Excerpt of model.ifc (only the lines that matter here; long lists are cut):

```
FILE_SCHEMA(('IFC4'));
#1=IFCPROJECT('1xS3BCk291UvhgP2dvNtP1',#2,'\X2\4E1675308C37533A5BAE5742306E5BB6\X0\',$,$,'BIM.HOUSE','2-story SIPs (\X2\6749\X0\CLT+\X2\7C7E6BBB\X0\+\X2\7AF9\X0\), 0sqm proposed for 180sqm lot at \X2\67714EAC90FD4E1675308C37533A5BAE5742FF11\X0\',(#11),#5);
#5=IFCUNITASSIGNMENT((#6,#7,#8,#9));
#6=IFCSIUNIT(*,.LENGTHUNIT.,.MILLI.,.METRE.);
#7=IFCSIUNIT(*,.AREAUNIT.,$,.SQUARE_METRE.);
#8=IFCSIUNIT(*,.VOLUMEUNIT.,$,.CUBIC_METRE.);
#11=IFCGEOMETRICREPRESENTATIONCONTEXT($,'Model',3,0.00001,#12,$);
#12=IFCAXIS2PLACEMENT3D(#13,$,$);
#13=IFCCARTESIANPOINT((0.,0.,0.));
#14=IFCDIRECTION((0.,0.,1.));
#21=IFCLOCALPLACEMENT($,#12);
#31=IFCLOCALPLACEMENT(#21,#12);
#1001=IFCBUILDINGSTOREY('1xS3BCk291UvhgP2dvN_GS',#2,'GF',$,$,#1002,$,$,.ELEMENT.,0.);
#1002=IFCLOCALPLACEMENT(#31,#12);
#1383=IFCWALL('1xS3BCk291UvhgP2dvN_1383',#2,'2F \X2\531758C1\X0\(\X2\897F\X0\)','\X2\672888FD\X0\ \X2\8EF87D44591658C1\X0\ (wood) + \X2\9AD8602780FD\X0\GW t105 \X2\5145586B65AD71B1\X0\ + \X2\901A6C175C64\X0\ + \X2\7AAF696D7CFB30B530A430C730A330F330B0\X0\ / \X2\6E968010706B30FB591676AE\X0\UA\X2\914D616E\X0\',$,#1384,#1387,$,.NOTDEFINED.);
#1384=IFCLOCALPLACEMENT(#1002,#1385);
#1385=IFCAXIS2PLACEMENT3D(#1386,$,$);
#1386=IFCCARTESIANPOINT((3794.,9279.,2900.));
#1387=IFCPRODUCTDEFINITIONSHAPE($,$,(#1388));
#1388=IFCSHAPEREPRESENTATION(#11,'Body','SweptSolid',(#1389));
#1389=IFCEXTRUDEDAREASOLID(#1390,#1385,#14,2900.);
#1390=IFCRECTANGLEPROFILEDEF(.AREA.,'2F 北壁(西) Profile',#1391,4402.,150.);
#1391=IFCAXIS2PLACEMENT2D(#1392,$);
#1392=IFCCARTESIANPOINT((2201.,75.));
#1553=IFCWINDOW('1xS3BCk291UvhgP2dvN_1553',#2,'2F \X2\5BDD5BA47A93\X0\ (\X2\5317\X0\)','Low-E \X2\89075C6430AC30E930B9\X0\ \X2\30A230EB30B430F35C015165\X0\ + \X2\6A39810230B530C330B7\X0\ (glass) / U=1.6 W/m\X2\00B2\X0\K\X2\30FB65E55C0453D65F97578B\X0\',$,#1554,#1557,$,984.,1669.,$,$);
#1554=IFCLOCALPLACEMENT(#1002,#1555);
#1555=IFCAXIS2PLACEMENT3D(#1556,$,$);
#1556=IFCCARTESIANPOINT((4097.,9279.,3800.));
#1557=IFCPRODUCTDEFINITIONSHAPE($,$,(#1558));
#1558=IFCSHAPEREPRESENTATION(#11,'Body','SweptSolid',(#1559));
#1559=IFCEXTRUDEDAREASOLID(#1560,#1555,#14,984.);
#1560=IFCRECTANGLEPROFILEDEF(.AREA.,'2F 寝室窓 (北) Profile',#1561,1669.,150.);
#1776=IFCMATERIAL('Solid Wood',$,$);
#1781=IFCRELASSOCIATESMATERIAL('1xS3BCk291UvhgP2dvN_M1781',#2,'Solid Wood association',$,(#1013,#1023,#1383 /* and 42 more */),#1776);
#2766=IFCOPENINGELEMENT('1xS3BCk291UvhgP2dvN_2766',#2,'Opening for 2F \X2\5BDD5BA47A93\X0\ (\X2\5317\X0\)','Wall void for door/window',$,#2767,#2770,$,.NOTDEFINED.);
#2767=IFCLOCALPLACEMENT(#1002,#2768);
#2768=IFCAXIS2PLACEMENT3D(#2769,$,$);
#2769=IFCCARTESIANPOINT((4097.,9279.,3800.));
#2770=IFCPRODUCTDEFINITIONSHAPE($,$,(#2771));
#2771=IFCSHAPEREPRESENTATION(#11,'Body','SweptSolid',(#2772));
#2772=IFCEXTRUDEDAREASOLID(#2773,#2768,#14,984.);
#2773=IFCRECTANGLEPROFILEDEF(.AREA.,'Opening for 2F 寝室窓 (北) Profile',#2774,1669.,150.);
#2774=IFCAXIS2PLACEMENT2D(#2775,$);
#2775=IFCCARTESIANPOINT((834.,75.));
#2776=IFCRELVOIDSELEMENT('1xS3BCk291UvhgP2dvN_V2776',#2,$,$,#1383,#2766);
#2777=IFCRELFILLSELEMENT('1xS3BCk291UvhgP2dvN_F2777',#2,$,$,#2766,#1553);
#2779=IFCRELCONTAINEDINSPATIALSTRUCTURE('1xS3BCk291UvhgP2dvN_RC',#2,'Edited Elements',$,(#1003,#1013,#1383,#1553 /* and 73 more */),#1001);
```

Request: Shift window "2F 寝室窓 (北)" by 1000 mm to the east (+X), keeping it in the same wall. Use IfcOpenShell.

```python
import ifcopenshell
import ifcopenshell.api.geometry
import ifcopenshell.util.placement
import ifcopenshell.util.unit

model = ifcopenshell.open("model.ifc")
unit_scale = ifcopenshell.util.unit.calculate_unit_scale(model)

window = model.by_guid("1xS3BCk291UvhgP2dvN_1553")
opening = window.FillsVoids[0].RelatingOpeningElement
wall = opening.VoidsElements[0].RelatingBuildingElement

wall_matrix = ifcopenshell.util.placement.get_local_placement(wall.ObjectPlacement)
shift = wall_matrix[:3, 0] * 1 / unit_scale
before = ifcopenshell.util.placement.get_local_placement(window.ObjectPlacement)[:3, 3].copy()

# The window is not placed relative to its opening, so move both.
for product in (opening, window):
    matrix = ifcopenshell.util.placement.get_local_placement(product.ObjectPlacement)
    matrix[:3, 3] += shift
    ifcopenshell.api.geometry.edit_object_placement(model, product=product, matrix=matrix, is_si=False)

after = ifcopenshell.util.placement.get_local_placement(window.ObjectPlacement)[:3, 3]
print("window moved by", (after - before).round(3) + 0.0)

model.write("model-out.ifc")
```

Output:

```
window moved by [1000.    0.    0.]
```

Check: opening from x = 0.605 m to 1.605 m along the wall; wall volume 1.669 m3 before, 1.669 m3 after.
